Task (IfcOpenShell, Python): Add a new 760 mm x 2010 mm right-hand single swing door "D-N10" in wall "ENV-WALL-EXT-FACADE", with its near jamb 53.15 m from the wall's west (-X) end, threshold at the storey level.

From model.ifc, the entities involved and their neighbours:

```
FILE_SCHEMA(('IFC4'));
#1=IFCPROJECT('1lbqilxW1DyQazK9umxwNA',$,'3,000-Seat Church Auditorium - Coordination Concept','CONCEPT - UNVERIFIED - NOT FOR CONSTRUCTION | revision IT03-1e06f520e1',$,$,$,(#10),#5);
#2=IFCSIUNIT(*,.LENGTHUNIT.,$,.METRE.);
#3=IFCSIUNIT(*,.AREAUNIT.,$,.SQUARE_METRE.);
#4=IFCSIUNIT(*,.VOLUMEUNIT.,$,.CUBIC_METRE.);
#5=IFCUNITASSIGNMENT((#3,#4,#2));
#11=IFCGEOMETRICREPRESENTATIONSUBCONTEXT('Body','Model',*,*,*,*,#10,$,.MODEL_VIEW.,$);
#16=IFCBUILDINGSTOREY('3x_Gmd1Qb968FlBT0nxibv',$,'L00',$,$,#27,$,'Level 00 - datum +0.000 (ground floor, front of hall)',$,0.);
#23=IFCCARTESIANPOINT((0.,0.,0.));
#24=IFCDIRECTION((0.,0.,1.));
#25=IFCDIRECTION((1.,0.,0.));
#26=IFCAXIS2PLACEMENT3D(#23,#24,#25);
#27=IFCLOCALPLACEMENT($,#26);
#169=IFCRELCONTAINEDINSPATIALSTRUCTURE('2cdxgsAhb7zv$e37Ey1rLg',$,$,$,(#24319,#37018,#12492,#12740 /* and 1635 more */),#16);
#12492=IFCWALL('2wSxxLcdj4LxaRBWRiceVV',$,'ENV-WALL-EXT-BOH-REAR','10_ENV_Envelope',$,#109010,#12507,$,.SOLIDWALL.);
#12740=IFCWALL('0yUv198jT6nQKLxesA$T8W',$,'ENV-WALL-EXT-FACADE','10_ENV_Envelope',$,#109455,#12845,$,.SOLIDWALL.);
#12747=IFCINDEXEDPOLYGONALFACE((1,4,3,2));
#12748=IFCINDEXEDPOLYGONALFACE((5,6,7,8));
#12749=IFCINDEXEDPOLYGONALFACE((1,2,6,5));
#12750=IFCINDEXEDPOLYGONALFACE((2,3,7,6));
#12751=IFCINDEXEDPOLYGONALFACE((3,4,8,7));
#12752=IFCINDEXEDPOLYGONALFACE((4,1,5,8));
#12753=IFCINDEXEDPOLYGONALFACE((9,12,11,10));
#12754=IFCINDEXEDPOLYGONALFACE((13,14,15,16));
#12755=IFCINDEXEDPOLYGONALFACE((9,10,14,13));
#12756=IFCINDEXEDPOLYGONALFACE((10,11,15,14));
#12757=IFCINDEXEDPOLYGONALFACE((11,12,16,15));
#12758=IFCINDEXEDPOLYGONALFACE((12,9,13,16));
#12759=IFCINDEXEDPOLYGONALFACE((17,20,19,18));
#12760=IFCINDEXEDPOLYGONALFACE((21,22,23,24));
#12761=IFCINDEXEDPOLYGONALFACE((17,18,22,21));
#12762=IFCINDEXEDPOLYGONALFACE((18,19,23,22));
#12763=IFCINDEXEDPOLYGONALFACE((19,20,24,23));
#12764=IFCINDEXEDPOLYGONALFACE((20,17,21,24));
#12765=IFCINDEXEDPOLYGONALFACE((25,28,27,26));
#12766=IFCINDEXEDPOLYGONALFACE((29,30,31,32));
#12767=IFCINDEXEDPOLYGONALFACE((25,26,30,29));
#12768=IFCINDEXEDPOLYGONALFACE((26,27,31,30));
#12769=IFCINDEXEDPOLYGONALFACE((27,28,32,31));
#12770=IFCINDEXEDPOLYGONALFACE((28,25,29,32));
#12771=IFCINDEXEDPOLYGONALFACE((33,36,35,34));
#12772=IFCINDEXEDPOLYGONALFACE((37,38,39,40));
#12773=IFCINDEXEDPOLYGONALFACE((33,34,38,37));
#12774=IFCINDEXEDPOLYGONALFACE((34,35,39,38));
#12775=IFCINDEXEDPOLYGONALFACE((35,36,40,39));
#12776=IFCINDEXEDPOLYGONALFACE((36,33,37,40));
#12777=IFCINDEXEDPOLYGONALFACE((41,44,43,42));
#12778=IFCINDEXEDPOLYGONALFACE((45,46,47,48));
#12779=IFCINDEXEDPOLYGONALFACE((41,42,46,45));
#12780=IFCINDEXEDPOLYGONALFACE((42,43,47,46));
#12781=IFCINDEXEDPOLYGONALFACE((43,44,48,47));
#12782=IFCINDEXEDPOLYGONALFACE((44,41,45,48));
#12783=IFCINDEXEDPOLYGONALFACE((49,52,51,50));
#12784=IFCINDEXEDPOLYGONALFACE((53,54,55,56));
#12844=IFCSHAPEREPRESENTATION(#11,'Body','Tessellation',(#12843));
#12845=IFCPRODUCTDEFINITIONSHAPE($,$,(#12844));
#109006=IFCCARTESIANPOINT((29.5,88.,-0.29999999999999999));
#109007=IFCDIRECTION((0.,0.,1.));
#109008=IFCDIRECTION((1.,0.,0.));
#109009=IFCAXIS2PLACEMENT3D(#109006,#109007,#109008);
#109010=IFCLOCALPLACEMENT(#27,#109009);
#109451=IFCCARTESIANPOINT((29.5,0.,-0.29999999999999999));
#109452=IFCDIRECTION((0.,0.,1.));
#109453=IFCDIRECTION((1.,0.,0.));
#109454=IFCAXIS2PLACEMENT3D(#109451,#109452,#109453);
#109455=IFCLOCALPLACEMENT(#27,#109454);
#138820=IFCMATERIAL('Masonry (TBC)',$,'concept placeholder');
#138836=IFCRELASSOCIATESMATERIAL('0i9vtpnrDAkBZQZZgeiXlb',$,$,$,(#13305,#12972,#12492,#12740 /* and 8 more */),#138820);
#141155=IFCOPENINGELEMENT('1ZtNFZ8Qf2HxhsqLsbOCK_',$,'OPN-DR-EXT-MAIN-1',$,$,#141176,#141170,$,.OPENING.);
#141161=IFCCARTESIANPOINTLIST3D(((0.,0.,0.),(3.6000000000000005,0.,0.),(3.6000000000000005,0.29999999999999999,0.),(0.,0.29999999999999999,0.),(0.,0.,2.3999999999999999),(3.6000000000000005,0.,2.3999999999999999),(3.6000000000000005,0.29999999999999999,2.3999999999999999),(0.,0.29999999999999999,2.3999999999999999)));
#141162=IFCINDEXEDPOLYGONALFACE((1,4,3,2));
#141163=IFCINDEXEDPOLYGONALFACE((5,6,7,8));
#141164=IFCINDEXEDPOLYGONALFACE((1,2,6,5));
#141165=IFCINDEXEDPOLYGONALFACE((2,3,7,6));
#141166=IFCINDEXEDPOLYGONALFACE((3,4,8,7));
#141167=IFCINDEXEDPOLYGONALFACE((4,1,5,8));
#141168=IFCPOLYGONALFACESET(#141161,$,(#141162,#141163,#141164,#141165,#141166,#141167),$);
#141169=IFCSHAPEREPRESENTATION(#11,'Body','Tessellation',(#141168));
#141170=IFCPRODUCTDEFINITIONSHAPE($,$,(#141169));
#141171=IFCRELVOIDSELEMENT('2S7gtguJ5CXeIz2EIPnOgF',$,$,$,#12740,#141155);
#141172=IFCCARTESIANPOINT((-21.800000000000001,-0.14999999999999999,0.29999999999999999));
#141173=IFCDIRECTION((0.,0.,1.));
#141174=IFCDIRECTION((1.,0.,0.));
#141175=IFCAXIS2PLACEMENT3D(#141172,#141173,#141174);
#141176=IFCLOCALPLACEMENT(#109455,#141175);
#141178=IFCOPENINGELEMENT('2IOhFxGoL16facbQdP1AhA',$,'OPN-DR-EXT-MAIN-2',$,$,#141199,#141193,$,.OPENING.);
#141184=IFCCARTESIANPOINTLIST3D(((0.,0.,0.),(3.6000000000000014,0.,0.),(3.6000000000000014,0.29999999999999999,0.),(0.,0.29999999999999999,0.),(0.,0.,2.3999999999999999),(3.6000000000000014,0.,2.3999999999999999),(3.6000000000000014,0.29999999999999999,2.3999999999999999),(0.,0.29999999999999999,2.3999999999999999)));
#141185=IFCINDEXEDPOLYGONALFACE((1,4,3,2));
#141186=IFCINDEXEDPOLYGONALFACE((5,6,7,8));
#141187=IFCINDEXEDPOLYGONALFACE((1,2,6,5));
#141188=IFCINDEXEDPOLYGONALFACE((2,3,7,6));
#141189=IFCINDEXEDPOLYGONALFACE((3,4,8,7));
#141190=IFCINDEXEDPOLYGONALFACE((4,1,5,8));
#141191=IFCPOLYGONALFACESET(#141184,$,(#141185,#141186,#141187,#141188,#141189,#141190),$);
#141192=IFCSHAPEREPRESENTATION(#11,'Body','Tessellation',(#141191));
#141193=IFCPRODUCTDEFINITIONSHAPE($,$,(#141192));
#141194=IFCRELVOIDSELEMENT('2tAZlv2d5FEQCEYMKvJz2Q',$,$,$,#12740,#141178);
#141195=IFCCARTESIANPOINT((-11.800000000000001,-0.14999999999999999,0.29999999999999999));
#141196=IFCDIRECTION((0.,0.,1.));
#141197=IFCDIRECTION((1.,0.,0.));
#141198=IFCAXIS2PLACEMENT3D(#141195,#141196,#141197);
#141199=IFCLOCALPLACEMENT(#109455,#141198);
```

```python
import numpy as np
import ifcopenshell
import ifcopenshell.api.feature
import ifcopenshell.api.geometry
import ifcopenshell.api.root
import ifcopenshell.api.spatial
import ifcopenshell.geom
import ifcopenshell.util.element
import ifcopenshell.util.placement
import ifcopenshell.util.representation
import ifcopenshell.util.shape
import ifcopenshell.util.unit

model = ifcopenshell.open("model.ifc")
unit_scale = ifcopenshell.util.unit.calculate_unit_scale(model)
settings = ifcopenshell.geom.settings()


def volume(element):
    """Net volume in cubic metres, openings subtracted."""
    shape = ifcopenshell.geom.create_shape(settings, element)
    return ifcopenshell.util.shape.get_volume(shape.geometry)


wall = model.by_guid("0yUv198jT6nQKLxesA$T8W")
storey = ifcopenshell.util.element.get_container(wall, ifc_class="IfcBuildingStorey")
context = ifcopenshell.util.representation.get_context(model, "Model", "Body", "MODEL_VIEW")
before = volume(wall)

width, height, from_end, sill = 0.76, 2.01, 53.15, 0.0  # metres

# The wall runs along its own X axis, and the end named is its -X end.
wall_shape = ifcopenshell.geom.create_shape(settings, wall)
x, y, z = ifcopenshell.util.shape.get_vertices(wall_shape.geometry).T
start = x.min() + from_end
face, thickness = float(y.min()), float(y.max() - y.min())
wall_matrix = ifcopenshell.util.placement.get_local_placement(wall.ObjectPlacement)
level = ifcopenshell.util.placement.get_local_placement(storey.ObjectPlacement)[2, 3]


def in_wall(x, y):
    """Placement at x, y metres in the wall's axes, at sill height."""
    matrix = wall_matrix.copy()
    matrix[:, 3] = wall_matrix @ np.array([x / unit_scale, y / unit_scale, 0.0, 1.0])
    matrix[2, 3] = level + sill / unit_scale
    return matrix


# Opening: a box that overshoots both wall faces by 50 mm.
opening = ifcopenshell.api.root.create_entity(model, ifc_class="IfcOpeningElement", predefined_type="OPENING")
box = ifcopenshell.api.geometry.add_wall_representation(
    model, context=context, length=width, height=height, thickness=thickness + 0.1
)
ifcopenshell.api.geometry.assign_representation(model, product=opening, representation=box)
ifcopenshell.api.geometry.edit_object_placement(model, product=opening, matrix=in_wall(start, face - 0.05), is_si=False)
ifcopenshell.api.feature.add_feature(model, feature=opening, element=wall)

door = ifcopenshell.api.root.create_entity(model, ifc_class="IfcDoor", name="D-N10", predefined_type="DOOR")
door.OverallWidth, door.OverallHeight = width / unit_scale, height / unit_scale
door.OperationType = "SINGLE_SWING_RIGHT"
body = ifcopenshell.api.geometry.add_door_representation(
    model,
    context=context,
    overall_width=door.OverallWidth,
    overall_height=door.OverallHeight,
    operation_type="SINGLE_SWING_RIGHT",
    lining_properties={"LiningDepth": thickness / unit_scale, "ThresholdDepth": thickness / unit_scale},
)
ifcopenshell.api.geometry.assign_representation(model, product=door, representation=body)
ifcopenshell.api.spatial.assign_container(model, products=[door], relating_structure=storey)
ifcopenshell.api.feature.add_filling(model, opening=opening, element=door)

# The lining spans the wall, so the door starts at the wall face.
ifcopenshell.api.geometry.edit_object_placement(model, product=door, matrix=in_wall(start, face), is_si=False)

after = volume(wall)

print(f"wall volume {before:.3f} -> {after:.3f} m3")

model.write("model-out.ifc")
```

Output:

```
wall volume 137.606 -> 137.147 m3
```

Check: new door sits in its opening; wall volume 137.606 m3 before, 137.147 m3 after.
